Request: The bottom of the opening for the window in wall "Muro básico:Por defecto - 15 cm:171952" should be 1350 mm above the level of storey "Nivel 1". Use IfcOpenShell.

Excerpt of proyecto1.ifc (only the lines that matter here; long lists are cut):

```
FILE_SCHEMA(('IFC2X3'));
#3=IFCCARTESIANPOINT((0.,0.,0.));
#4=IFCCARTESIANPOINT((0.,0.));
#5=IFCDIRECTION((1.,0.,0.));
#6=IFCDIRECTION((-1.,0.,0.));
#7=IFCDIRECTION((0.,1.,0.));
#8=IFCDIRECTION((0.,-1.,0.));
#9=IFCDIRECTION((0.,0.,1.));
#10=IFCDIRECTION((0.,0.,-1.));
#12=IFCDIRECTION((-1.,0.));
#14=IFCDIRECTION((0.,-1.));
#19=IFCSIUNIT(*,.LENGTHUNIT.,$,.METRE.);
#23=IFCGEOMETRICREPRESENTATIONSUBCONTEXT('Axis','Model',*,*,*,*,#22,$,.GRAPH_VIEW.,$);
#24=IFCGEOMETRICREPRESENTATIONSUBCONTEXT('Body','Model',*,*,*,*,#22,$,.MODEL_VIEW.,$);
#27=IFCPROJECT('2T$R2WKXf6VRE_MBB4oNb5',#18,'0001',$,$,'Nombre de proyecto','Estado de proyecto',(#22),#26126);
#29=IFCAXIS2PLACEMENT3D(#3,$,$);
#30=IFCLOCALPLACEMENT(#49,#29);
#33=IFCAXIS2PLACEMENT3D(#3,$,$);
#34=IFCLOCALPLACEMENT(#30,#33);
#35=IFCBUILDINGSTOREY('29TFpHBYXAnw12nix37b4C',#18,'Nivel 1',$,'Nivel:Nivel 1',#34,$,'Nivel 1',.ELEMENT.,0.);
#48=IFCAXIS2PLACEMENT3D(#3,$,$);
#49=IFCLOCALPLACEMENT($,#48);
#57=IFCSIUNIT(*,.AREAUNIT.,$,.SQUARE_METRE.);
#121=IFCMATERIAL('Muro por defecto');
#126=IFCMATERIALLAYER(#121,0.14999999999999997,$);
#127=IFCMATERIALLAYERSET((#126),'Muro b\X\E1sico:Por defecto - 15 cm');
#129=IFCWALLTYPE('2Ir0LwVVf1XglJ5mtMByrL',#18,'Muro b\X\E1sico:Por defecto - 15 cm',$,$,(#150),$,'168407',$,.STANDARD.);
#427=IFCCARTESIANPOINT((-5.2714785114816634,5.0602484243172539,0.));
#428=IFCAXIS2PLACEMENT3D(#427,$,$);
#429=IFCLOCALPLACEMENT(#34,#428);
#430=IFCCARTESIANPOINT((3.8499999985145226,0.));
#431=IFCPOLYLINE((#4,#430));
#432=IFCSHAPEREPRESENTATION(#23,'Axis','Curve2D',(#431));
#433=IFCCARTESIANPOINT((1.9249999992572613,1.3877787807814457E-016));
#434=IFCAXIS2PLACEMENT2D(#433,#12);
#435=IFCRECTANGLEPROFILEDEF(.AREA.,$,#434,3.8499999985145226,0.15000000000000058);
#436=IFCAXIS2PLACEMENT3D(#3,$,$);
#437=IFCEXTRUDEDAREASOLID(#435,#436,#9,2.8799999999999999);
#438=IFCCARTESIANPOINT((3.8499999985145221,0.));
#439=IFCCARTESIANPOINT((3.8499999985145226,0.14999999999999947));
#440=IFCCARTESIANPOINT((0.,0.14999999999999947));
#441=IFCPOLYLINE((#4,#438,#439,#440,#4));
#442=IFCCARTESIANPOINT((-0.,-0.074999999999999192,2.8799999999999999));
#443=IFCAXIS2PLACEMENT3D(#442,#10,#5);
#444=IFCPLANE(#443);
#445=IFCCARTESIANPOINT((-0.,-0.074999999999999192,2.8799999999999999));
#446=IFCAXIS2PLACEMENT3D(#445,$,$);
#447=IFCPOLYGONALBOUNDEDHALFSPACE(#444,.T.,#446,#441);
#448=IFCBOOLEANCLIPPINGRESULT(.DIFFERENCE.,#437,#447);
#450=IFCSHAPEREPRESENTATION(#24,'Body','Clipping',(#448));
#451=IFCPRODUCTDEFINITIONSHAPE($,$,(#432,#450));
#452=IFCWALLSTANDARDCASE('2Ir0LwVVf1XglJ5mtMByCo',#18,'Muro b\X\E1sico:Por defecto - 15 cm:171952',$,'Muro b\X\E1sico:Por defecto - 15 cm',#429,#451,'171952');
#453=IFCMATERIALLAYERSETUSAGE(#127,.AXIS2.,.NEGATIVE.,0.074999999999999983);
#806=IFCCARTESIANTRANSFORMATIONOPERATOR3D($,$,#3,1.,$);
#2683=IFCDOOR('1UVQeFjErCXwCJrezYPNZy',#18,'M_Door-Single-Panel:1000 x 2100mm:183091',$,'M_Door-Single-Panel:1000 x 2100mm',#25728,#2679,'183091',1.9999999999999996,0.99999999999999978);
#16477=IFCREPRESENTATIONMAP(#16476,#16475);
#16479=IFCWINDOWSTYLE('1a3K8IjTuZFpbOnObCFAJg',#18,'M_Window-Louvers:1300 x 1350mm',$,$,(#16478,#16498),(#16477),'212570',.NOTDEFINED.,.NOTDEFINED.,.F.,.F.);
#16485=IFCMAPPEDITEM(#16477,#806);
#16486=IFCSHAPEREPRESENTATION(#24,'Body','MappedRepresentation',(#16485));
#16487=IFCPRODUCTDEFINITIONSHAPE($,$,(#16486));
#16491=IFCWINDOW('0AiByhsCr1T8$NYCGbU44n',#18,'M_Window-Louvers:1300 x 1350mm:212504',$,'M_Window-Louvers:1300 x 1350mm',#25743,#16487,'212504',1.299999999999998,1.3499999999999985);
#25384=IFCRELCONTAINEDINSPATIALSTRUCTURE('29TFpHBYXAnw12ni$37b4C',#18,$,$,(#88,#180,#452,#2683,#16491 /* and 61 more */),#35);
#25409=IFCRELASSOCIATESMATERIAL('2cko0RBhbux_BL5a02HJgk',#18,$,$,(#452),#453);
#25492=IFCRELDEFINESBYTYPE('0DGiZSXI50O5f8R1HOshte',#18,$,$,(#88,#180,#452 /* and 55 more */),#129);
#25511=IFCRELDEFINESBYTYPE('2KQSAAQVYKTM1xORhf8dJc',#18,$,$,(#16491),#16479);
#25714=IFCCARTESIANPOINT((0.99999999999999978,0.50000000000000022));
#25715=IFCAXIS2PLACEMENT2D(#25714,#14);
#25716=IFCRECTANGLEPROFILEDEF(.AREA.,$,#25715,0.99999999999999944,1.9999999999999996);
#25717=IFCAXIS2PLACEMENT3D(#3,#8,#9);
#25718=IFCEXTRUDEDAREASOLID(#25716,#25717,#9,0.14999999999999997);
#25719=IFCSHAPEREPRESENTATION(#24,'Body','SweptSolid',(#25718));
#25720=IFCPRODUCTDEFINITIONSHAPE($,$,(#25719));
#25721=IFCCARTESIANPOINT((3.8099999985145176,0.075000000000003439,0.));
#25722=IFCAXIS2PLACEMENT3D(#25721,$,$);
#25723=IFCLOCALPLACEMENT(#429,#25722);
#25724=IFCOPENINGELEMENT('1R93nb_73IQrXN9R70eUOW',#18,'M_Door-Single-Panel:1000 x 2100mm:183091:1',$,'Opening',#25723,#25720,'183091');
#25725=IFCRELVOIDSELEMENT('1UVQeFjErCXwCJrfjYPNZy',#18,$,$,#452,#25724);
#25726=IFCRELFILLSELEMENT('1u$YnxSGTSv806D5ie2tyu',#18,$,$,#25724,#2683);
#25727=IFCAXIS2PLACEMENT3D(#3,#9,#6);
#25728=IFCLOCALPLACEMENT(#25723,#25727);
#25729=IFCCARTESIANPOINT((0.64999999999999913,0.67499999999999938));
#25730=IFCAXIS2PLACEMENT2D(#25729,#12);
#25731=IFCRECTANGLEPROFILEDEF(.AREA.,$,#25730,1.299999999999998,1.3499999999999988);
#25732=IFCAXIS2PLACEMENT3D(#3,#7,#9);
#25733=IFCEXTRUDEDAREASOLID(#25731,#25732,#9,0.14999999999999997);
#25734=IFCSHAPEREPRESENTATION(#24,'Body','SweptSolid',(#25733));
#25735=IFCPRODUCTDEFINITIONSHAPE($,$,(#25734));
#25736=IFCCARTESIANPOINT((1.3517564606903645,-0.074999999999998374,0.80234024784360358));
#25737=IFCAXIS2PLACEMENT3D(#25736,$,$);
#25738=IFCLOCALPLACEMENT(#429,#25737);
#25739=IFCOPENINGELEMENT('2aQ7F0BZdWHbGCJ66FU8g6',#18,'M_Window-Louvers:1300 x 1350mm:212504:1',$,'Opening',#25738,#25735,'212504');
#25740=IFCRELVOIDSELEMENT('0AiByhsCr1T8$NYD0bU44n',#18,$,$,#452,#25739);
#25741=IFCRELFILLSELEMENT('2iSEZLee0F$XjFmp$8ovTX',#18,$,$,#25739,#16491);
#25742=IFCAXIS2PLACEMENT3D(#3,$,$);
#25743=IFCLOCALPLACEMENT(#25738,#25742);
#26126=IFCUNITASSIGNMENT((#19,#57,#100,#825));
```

```python
import numpy as np
import ifcopenshell
import ifcopenshell.api.geometry
import ifcopenshell.geom
import ifcopenshell.util.element
import ifcopenshell.util.placement
import ifcopenshell.util.shape
import ifcopenshell.util.unit

model = ifcopenshell.open("proyecto1.ifc")
unit_scale = ifcopenshell.util.unit.calculate_unit_scale(model)

window = model.by_guid("0AiByhsCr1T8$NYCGbU44n")
opening = window.FillsVoids[0].RelatingOpeningElement
storey = ifcopenshell.util.element.get_container(window, ifc_class="IfcBuildingStorey")
level = ifcopenshell.util.placement.get_local_placement(storey.ObjectPlacement)[2, 3]

# The opening's origin need not be at the sill, so measure its lowest point.
shape = ifcopenshell.geom.create_shape(ifcopenshell.geom.settings(), opening)
bottom = ifcopenshell.util.shape.get_shape_bottom_elevation(shape, shape.geometry) / unit_scale
dz = level + 1.35 / unit_scale - bottom

shift = np.array([0.0, 0.0, dz])
# The window is placed relative to its opening, so it follows when the opening moves.
matrix = ifcopenshell.util.placement.get_local_placement(opening.ObjectPlacement)
matrix[:3, 3] += shift
ifcopenshell.api.geometry.edit_object_placement(
    model, product=opening, matrix=matrix, is_si=False, should_transform_children=True
)

print(f"moved by {dz * unit_scale:+.3f} m")

model.write("proyecto1_v2.ifc")
```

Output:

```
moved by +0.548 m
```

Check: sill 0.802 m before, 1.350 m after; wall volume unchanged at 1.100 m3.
